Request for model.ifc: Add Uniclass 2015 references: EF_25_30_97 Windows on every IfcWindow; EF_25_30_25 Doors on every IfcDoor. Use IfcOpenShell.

First a look at what the model holds.

```python
import ifcopenshell

model = ifcopenshell.open("model.ifc")
print(model.schema)
print("classifications:", [c.Name for c in model.by_type("IfcClassification")])
for ifc_class in ("IfcDoor", "IfcRoof", "IfcStair", "IfcWall", "IfcWindow"):
    print(ifc_class, len(model.by_type(ifc_class)))
```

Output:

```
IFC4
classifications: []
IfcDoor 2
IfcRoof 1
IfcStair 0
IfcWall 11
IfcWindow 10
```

```python
import ifcopenshell
import ifcopenshell.api.classification

model = ifcopenshell.open("model.ifc")

system = ifcopenshell.api.classification.add_classification(model, classification="Uniclass 2015")

codes = {
    "IfcWindow": ("EF_25_30_97", "Windows"),
    "IfcDoor": ("EF_25_30_25", "Doors"),
}
for ifc_class, (code, name) in codes.items():
    products = model.by_type(ifc_class)
    ifcopenshell.api.classification.add_reference(
        model, products=products, classification=system, identification=code, name=name
    )
    print(code, len(products))

model.write("model_rev.ifc")
```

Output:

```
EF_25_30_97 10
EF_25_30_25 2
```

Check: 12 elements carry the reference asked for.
